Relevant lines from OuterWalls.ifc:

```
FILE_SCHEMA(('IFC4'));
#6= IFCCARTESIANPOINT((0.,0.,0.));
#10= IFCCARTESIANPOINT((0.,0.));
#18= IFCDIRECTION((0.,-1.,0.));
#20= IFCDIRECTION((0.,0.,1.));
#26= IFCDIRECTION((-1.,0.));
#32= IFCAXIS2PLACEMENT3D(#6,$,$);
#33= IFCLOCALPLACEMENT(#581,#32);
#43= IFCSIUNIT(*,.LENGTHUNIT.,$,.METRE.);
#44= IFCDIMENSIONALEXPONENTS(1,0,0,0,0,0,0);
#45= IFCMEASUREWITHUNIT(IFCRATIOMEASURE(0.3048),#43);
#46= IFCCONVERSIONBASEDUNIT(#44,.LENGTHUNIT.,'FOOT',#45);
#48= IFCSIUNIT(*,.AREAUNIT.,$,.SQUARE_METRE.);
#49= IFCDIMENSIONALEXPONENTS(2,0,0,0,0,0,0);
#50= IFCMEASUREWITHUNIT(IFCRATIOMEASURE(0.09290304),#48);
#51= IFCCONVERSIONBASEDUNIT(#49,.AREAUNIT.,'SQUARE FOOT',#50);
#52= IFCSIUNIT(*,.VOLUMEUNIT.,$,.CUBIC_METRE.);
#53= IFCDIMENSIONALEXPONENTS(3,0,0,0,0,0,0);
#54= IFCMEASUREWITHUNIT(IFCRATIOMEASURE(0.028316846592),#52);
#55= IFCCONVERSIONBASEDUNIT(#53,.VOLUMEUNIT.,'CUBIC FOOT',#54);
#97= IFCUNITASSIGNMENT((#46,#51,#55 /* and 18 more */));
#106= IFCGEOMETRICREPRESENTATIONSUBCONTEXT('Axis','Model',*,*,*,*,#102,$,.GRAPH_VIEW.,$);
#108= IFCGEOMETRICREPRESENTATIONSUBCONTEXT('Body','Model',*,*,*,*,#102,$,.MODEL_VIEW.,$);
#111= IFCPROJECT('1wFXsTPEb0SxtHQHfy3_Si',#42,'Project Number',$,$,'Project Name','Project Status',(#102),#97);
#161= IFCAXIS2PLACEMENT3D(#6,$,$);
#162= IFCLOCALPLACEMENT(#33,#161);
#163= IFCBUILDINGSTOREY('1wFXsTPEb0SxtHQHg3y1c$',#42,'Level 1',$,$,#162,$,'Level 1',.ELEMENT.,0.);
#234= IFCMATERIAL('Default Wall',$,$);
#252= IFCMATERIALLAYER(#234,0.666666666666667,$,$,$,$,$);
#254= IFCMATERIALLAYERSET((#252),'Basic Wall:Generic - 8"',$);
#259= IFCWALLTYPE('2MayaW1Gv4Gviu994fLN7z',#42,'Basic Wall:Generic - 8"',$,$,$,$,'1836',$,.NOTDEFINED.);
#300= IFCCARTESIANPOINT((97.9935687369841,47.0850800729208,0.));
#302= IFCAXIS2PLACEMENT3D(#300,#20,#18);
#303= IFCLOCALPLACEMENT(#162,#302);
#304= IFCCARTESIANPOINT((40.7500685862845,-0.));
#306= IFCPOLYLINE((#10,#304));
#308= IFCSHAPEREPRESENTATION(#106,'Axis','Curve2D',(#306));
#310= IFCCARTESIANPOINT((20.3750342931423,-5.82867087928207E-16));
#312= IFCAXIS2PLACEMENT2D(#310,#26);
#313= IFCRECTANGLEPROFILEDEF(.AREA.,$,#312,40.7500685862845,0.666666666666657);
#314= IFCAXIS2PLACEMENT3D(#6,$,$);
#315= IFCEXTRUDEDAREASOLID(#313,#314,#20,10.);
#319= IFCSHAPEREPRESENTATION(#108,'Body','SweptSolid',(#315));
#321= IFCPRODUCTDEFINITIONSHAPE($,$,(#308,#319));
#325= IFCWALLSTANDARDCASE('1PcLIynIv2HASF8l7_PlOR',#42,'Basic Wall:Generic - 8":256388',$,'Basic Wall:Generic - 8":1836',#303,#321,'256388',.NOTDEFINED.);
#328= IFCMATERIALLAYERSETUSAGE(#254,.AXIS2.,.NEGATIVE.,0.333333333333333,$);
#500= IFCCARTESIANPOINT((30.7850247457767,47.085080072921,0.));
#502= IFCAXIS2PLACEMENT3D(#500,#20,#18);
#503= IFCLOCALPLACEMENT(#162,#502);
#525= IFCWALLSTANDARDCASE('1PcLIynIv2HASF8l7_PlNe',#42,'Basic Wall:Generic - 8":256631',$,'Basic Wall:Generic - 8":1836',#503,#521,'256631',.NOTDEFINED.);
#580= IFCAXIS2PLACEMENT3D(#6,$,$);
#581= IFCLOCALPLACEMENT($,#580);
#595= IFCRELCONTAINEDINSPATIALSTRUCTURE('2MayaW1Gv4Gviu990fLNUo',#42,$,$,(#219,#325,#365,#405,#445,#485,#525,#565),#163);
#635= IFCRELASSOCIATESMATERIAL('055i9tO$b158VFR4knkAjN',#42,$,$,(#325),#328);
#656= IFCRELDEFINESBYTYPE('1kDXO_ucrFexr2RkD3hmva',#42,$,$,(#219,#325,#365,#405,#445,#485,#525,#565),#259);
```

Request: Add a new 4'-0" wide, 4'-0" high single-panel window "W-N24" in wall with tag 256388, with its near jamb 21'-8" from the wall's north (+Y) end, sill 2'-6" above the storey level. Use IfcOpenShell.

```python
import numpy as np
import ifcopenshell
import ifcopenshell.api.feature
import ifcopenshell.api.geometry
import ifcopenshell.api.root
import ifcopenshell.api.spatial
import ifcopenshell.geom
import ifcopenshell.util.element
import ifcopenshell.util.placement
import ifcopenshell.util.representation
import ifcopenshell.util.shape
import ifcopenshell.util.unit

model = ifcopenshell.open("OuterWalls.ifc")
unit_scale = ifcopenshell.util.unit.calculate_unit_scale(model)
settings = ifcopenshell.geom.settings()


def volume(element):
    """Net volume in cubic metres, openings subtracted."""
    shape = ifcopenshell.geom.create_shape(settings, element)
    return ifcopenshell.util.shape.get_volume(shape.geometry)


wall = model.by_guid("1PcLIynIv2HASF8l7_PlOR")
storey = ifcopenshell.util.element.get_container(wall, ifc_class="IfcBuildingStorey")
context = ifcopenshell.util.representation.get_context(model, "Model", "Body", "MODEL_VIEW")
before = volume(wall)

width, height, from_end, sill = 1.2192, 1.2192, 6.604, 0.762  # metres

# The wall runs along its own X axis, and the end named is its -X end.
wall_shape = ifcopenshell.geom.create_shape(settings, wall)
x, y, z = ifcopenshell.util.shape.get_vertices(wall_shape.geometry).T
start = x.min() + from_end
face, thickness = float(y.min()), float(y.max() - y.min())
wall_matrix = ifcopenshell.util.placement.get_local_placement(wall.ObjectPlacement)
level = ifcopenshell.util.placement.get_local_placement(storey.ObjectPlacement)[2, 3]


def in_wall(x, y):
    """Placement at x, y metres in the wall's axes, at sill height."""
    matrix = wall_matrix.copy()
    matrix[:, 3] = wall_matrix @ np.array([x / unit_scale, y / unit_scale, 0.0, 1.0])
    matrix[2, 3] = level + sill / unit_scale
    return matrix


# Opening: a box that overshoots both wall faces by 50 mm.
opening = ifcopenshell.api.root.create_entity(model, ifc_class="IfcOpeningElement", predefined_type="OPENING")
box = ifcopenshell.api.geometry.add_wall_representation(
    model, context=context, length=width, height=height, thickness=thickness + 0.1
)
ifcopenshell.api.geometry.assign_representation(model, product=opening, representation=box)
ifcopenshell.api.geometry.edit_object_placement(model, product=opening, matrix=in_wall(start, face - 0.05), is_si=False)
ifcopenshell.api.feature.add_feature(model, feature=opening, element=wall)

window = ifcopenshell.api.root.create_entity(model, ifc_class="IfcWindow", name="W-N24", predefined_type="WINDOW")
window.OverallWidth, window.OverallHeight = width / unit_scale, height / unit_scale
window.PartitioningType = "SINGLE_PANEL"
body = ifcopenshell.api.geometry.add_window_representation(
    model,
    context=context,
    overall_width=window.OverallWidth,
    overall_height=window.OverallHeight,
    partition_type="SINGLE_PANEL",
)
ifcopenshell.api.geometry.assign_representation(model, product=window, representation=body)
ifcopenshell.api.spatial.assign_container(model, products=[window], relating_structure=storey)
ifcopenshell.api.feature.add_filling(model, opening=opening, element=window)

# Centre the window in the wall's thickness.
ifcopenshell.api.geometry.edit_object_placement(model, product=window, matrix=in_wall(start, face), is_si=False)
window_shape = ifcopenshell.geom.create_shape(settings, window)
depth = ifcopenshell.util.shape.get_vertices(window_shape.geometry)[:, 1]
offset = face + thickness / 2 - (depth.min() + depth.max()) / 2
ifcopenshell.api.geometry.edit_object_placement(model, product=window, matrix=in_wall(start, offset), is_si=False)

after = volume(wall)

print(f"wall volume {before:.3f} -> {after:.3f} m3")

model.write("OuterWalls_updated.ifc")
```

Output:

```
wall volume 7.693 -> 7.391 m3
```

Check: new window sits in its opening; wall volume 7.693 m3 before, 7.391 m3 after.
